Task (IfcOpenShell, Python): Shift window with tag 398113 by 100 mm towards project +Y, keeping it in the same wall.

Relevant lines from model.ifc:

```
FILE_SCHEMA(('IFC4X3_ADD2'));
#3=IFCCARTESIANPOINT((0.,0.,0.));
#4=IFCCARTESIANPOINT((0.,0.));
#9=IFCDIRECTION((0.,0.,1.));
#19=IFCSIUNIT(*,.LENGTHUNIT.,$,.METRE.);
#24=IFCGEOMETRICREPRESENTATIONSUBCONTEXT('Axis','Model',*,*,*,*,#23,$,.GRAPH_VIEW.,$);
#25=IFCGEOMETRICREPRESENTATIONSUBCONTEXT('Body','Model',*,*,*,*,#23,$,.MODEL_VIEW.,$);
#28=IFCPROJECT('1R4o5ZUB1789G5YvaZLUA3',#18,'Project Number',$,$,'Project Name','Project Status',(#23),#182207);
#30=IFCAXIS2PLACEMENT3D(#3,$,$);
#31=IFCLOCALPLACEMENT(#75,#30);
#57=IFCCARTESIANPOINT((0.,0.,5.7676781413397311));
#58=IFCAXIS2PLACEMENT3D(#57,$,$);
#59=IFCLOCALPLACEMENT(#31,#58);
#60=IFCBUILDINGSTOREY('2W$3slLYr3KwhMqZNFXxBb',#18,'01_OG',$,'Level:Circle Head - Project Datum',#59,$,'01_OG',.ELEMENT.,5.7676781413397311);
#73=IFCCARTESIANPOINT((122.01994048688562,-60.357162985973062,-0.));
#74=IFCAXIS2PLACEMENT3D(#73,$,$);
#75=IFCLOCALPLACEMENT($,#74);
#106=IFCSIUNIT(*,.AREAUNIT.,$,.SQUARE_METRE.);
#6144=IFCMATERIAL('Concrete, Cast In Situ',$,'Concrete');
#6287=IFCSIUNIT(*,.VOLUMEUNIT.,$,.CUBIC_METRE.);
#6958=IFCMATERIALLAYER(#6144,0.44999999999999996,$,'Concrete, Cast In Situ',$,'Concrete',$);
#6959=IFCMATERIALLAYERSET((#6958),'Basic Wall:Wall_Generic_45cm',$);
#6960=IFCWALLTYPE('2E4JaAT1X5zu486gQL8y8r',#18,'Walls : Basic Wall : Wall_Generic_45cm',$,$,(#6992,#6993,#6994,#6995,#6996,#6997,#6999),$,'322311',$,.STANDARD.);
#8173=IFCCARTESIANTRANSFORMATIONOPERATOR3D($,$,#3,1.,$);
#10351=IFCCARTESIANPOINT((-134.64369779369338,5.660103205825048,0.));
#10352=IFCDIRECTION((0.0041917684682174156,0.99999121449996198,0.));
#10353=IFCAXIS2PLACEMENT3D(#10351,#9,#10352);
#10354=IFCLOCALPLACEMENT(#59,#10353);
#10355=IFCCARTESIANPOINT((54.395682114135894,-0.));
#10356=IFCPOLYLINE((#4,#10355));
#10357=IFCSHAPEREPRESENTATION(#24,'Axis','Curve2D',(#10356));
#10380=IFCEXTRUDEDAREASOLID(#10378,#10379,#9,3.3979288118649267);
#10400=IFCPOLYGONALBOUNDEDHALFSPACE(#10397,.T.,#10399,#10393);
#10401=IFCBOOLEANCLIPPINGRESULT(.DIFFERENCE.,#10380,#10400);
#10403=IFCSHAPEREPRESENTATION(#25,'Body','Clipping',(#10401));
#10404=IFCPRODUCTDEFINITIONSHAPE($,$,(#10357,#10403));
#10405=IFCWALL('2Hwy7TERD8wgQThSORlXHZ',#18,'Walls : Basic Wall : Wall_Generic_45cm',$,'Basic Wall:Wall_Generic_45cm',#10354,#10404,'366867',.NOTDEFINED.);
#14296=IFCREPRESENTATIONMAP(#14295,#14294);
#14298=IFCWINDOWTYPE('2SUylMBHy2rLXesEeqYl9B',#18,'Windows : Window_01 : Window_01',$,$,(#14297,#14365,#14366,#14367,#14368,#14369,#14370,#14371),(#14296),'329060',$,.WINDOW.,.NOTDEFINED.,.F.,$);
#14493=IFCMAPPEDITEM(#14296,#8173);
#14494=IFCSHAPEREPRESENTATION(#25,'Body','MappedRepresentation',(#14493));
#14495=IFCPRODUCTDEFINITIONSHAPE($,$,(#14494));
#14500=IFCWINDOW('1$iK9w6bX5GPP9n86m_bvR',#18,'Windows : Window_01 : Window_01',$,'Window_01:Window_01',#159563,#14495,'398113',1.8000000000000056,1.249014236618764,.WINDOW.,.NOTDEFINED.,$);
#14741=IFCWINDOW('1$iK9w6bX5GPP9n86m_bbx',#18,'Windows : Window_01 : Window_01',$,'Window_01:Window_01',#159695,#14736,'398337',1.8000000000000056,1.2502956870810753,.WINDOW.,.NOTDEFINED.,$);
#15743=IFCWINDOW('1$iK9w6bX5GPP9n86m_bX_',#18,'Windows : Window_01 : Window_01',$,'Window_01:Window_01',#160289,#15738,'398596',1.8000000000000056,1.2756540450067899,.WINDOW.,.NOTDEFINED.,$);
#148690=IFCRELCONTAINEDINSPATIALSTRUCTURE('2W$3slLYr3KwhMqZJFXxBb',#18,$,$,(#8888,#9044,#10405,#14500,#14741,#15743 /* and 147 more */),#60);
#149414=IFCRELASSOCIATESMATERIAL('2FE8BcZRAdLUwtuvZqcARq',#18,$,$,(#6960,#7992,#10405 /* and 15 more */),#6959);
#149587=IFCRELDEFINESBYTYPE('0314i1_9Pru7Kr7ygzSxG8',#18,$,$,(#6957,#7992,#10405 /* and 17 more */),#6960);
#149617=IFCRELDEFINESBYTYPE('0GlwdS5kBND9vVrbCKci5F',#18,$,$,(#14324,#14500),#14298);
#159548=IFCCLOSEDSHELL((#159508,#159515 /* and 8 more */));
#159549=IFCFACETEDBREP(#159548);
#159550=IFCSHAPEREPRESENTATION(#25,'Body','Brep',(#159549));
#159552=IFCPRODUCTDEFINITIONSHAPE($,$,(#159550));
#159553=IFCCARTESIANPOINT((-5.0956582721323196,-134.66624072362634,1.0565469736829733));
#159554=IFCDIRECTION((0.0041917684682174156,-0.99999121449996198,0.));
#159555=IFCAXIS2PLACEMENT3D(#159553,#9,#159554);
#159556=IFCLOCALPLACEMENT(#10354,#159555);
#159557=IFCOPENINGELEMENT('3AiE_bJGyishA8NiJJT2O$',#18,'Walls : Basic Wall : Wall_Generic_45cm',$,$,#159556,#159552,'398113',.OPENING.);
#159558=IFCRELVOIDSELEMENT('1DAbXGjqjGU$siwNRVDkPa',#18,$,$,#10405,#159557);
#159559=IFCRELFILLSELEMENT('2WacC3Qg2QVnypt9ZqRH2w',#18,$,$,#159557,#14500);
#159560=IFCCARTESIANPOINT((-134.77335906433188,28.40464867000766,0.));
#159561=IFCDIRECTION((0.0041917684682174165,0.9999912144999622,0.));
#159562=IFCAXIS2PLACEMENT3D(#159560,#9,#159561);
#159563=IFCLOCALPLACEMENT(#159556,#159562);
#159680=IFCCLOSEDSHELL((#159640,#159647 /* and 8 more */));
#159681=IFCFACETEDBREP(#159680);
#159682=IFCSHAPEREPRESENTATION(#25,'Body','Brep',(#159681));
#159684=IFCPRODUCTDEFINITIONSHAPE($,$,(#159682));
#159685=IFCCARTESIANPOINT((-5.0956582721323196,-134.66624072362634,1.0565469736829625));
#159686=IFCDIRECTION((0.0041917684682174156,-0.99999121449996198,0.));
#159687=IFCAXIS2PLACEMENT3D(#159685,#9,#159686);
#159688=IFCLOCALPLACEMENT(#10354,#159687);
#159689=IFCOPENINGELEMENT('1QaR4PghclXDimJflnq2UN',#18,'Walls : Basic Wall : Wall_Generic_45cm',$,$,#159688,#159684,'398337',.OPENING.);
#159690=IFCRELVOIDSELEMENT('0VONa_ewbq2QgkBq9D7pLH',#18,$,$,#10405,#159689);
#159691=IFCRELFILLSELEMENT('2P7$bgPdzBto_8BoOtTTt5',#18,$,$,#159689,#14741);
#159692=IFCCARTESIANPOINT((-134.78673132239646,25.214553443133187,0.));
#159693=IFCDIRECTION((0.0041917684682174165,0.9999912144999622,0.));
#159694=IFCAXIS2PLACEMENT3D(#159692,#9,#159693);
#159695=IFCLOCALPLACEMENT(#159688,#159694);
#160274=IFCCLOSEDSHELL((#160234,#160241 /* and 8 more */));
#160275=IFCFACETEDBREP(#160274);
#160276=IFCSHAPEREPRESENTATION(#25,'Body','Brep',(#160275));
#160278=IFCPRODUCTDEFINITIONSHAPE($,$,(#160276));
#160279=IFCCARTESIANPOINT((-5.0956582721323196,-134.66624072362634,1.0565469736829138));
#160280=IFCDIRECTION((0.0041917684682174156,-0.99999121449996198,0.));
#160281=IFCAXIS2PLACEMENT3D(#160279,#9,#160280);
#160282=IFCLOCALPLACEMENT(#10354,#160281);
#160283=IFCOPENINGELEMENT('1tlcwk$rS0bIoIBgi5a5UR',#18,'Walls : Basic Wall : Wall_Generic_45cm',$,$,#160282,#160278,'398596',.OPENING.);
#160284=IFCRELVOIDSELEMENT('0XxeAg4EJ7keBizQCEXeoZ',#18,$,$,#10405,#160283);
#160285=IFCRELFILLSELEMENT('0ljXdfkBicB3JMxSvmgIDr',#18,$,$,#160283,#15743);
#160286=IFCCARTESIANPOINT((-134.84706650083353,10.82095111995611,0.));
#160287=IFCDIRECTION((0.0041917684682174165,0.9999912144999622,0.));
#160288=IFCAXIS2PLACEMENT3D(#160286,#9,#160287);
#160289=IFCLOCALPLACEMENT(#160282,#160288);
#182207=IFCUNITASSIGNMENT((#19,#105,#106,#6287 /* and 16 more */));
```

```python
import ifcopenshell
import ifcopenshell.api.geometry
import ifcopenshell.util.placement
import ifcopenshell.util.unit

model = ifcopenshell.open("model.ifc")
unit_scale = ifcopenshell.util.unit.calculate_unit_scale(model)

window = model.by_id(14500)
opening = window.FillsVoids[0].RelatingOpeningElement
wall = opening.VoidsElements[0].RelatingBuildingElement

wall_matrix = ifcopenshell.util.placement.get_local_placement(wall.ObjectPlacement)
shift = wall_matrix[:3, 0] * 0.1 / unit_scale
before = ifcopenshell.util.placement.get_local_placement(window.ObjectPlacement)[:3, 3].copy()

# The window is placed relative to its opening, so it follows when the opening moves.
matrix = ifcopenshell.util.placement.get_local_placement(opening.ObjectPlacement)
matrix[:3, 3] += shift
ifcopenshell.api.geometry.edit_object_placement(
    model, product=opening, matrix=matrix, is_si=False, should_transform_children=True
)

after = ifcopenshell.util.placement.get_local_placement(window.ObjectPlacement)[:3, 3]
print("window moved by", (after - before).round(3) + 0.0)

model.write("model_rev.ifc")
```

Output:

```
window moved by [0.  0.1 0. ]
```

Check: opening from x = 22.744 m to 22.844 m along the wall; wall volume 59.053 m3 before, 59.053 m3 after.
